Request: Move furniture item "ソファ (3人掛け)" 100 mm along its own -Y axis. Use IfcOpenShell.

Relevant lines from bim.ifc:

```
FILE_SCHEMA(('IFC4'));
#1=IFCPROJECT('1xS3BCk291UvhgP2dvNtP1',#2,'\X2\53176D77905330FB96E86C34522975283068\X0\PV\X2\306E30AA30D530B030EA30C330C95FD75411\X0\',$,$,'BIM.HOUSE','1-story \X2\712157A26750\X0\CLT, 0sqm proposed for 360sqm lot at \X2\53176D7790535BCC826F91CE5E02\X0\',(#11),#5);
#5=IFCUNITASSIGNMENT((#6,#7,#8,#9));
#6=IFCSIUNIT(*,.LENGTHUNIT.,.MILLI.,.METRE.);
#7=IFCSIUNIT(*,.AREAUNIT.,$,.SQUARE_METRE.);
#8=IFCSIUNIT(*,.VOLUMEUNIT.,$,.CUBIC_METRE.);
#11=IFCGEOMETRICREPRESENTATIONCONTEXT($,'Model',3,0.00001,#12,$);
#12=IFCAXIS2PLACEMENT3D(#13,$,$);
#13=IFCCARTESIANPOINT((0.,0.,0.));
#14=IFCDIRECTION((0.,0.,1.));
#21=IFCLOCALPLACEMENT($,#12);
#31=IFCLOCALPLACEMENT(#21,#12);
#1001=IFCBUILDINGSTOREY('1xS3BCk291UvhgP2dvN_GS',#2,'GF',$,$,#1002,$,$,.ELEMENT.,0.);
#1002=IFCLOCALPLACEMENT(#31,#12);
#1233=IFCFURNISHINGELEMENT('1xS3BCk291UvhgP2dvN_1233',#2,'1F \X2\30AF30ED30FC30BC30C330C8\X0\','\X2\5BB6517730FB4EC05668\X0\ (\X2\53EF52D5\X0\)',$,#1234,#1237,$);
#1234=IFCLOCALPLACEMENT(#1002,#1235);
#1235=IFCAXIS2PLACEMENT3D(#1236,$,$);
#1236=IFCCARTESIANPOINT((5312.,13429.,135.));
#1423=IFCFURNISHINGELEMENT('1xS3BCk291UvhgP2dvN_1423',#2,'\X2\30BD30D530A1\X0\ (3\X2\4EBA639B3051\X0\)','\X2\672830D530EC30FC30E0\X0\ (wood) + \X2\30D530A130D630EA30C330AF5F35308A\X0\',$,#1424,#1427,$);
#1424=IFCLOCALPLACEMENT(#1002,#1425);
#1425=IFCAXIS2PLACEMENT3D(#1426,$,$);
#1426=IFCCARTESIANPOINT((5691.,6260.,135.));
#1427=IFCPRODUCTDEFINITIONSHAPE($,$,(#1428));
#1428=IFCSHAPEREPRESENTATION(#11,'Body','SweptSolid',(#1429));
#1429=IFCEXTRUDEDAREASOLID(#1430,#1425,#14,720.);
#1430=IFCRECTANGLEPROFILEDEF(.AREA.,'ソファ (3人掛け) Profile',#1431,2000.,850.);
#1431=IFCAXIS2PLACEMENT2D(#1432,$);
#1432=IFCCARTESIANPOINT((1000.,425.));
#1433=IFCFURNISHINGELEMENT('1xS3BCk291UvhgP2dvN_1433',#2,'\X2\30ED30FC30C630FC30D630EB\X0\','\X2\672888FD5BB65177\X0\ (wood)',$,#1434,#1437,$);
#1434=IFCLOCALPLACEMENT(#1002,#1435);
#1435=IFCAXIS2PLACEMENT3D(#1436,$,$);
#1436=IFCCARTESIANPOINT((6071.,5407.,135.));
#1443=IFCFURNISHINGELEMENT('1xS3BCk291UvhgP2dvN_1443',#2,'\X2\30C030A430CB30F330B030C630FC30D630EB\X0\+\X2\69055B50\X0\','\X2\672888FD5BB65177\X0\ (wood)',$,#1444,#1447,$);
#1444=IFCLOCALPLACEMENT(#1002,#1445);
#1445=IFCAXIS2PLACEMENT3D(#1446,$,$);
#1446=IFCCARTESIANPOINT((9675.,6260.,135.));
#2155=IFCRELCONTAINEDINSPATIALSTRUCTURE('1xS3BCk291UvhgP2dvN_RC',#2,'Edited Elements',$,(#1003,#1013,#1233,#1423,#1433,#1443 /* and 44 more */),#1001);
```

```python
import ifcopenshell
import ifcopenshell.api.geometry
import ifcopenshell.util.placement

model = ifcopenshell.open("bim.ifc")

item = model.by_guid("1xS3BCk291UvhgP2dvN_1423")
matrix = ifcopenshell.util.placement.get_local_placement(item.ObjectPlacement)
matrix[:3, 3] -= matrix[:3, 1] * 100.0
ifcopenshell.api.geometry.edit_object_placement(model, product=item, matrix=matrix, is_si=False)

print(ifcopenshell.util.placement.get_local_placement(item.ObjectPlacement).round(3) + 0.0)

model.write("bim_v2.ifc")
```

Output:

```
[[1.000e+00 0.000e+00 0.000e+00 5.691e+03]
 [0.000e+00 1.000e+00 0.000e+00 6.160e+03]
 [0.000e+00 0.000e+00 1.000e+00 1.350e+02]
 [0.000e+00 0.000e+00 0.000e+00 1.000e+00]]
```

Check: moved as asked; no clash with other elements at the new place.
